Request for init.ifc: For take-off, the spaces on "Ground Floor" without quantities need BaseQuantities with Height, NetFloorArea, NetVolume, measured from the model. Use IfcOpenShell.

First a look at what the model holds.

```python
import ifcopenshell
import ifcopenshell.util.element
import ifcopenshell.util.unit

model = ifcopenshell.open("init.ifc")
print(model.schema)
for unit_type in ("LENGTHUNIT", "AREAUNIT", "VOLUMEUNIT"):
    print(unit_type, ifcopenshell.util.unit.calculate_unit_scale(model, unit_type))
storey = next(s for s in model.by_type("IfcBuildingStorey") if s.Name == "Ground Floor")
spaces = [e for e in ifcopenshell.util.element.get_decomposition(storey) if e.is_a("IfcSpace")]
for e in sorted(spaces, key=lambda e: e.id()):
    print(e.id(), e.is_a(), e.Name, list(ifcopenshell.util.element.get_psets(e, qtos_only=True)), sep=" | ")
```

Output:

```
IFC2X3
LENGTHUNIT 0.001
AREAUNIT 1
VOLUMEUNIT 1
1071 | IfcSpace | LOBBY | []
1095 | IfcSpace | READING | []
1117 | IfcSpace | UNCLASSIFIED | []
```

```python
import ifcopenshell
import ifcopenshell.api.pset
import ifcopenshell.geom
import ifcopenshell.util.element
import ifcopenshell.util.shape
import ifcopenshell.util.unit

model = ifcopenshell.open("init.ifc")
unit_scale = ifcopenshell.util.unit.calculate_unit_scale(model)
area_scale = ifcopenshell.util.unit.calculate_unit_scale(model, "AREAUNIT")
volume_scale = ifcopenshell.util.unit.calculate_unit_scale(model, "VOLUMEUNIT")
settings = ifcopenshell.geom.settings()

storey = next(s for s in model.by_type("IfcBuildingStorey") if s.Name == "Ground Floor")
spaces = [e for e in ifcopenshell.util.element.get_decomposition(storey) if e.is_a("IfcSpace")]

for e in sorted(spaces, key=lambda e: e.id()):
    if ifcopenshell.util.element.get_psets(e, qtos_only=True, should_inherit=False):
        continue
    # Geometry comes back in metres, in the element's own axes.
    shape = ifcopenshell.geom.create_shape(settings, e)
    values = {
        "Height": ifcopenshell.util.shape.get_z(shape.geometry) / unit_scale,
        "NetFloorArea": ifcopenshell.util.shape.get_footprint_area(shape.geometry) / area_scale,
        "NetVolume": ifcopenshell.util.shape.get_volume(shape.geometry) / volume_scale,
    }
    qto = ifcopenshell.api.pset.add_qto(model, product=e, name="BaseQuantities")
    ifcopenshell.api.pset.edit_qto(model, qto=qto, properties=values)
    print(e.id(), {k: round(v, 3) for k, v in values.items()})

model.write("init_rev.ifc")
```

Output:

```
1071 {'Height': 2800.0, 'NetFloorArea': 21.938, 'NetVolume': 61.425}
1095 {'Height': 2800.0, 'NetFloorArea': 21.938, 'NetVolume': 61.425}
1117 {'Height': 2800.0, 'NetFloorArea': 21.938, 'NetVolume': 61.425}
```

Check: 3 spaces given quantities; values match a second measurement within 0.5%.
